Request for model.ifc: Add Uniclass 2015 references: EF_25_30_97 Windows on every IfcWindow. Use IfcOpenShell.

First a look at what the model holds.

```python
import ifcopenshell

model = ifcopenshell.open("model.ifc")
print(model.schema)
print("classifications:", [c.Name for c in model.by_type("IfcClassification")])
for ifc_class in ("IfcDoor", "IfcRoof", "IfcStair", "IfcWall", "IfcWindow"):
    print(ifc_class, len(model.by_type(ifc_class)))
```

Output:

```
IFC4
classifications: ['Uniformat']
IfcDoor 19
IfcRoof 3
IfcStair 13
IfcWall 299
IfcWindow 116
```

```python
import ifcopenshell
import ifcopenshell.api.classification

model = ifcopenshell.open("model.ifc")

system = ifcopenshell.api.classification.add_classification(model, classification="Uniclass 2015")

codes = {
    "IfcWindow": ("EF_25_30_97", "Windows"),
}
for ifc_class, (code, name) in codes.items():
    products = model.by_type(ifc_class)
    ifcopenshell.api.classification.add_reference(
        model, products=products, classification=system, identification=code, name=name
    )
    print(code, len(products))

model.write("model_updated.ifc")
```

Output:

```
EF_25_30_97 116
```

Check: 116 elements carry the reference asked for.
